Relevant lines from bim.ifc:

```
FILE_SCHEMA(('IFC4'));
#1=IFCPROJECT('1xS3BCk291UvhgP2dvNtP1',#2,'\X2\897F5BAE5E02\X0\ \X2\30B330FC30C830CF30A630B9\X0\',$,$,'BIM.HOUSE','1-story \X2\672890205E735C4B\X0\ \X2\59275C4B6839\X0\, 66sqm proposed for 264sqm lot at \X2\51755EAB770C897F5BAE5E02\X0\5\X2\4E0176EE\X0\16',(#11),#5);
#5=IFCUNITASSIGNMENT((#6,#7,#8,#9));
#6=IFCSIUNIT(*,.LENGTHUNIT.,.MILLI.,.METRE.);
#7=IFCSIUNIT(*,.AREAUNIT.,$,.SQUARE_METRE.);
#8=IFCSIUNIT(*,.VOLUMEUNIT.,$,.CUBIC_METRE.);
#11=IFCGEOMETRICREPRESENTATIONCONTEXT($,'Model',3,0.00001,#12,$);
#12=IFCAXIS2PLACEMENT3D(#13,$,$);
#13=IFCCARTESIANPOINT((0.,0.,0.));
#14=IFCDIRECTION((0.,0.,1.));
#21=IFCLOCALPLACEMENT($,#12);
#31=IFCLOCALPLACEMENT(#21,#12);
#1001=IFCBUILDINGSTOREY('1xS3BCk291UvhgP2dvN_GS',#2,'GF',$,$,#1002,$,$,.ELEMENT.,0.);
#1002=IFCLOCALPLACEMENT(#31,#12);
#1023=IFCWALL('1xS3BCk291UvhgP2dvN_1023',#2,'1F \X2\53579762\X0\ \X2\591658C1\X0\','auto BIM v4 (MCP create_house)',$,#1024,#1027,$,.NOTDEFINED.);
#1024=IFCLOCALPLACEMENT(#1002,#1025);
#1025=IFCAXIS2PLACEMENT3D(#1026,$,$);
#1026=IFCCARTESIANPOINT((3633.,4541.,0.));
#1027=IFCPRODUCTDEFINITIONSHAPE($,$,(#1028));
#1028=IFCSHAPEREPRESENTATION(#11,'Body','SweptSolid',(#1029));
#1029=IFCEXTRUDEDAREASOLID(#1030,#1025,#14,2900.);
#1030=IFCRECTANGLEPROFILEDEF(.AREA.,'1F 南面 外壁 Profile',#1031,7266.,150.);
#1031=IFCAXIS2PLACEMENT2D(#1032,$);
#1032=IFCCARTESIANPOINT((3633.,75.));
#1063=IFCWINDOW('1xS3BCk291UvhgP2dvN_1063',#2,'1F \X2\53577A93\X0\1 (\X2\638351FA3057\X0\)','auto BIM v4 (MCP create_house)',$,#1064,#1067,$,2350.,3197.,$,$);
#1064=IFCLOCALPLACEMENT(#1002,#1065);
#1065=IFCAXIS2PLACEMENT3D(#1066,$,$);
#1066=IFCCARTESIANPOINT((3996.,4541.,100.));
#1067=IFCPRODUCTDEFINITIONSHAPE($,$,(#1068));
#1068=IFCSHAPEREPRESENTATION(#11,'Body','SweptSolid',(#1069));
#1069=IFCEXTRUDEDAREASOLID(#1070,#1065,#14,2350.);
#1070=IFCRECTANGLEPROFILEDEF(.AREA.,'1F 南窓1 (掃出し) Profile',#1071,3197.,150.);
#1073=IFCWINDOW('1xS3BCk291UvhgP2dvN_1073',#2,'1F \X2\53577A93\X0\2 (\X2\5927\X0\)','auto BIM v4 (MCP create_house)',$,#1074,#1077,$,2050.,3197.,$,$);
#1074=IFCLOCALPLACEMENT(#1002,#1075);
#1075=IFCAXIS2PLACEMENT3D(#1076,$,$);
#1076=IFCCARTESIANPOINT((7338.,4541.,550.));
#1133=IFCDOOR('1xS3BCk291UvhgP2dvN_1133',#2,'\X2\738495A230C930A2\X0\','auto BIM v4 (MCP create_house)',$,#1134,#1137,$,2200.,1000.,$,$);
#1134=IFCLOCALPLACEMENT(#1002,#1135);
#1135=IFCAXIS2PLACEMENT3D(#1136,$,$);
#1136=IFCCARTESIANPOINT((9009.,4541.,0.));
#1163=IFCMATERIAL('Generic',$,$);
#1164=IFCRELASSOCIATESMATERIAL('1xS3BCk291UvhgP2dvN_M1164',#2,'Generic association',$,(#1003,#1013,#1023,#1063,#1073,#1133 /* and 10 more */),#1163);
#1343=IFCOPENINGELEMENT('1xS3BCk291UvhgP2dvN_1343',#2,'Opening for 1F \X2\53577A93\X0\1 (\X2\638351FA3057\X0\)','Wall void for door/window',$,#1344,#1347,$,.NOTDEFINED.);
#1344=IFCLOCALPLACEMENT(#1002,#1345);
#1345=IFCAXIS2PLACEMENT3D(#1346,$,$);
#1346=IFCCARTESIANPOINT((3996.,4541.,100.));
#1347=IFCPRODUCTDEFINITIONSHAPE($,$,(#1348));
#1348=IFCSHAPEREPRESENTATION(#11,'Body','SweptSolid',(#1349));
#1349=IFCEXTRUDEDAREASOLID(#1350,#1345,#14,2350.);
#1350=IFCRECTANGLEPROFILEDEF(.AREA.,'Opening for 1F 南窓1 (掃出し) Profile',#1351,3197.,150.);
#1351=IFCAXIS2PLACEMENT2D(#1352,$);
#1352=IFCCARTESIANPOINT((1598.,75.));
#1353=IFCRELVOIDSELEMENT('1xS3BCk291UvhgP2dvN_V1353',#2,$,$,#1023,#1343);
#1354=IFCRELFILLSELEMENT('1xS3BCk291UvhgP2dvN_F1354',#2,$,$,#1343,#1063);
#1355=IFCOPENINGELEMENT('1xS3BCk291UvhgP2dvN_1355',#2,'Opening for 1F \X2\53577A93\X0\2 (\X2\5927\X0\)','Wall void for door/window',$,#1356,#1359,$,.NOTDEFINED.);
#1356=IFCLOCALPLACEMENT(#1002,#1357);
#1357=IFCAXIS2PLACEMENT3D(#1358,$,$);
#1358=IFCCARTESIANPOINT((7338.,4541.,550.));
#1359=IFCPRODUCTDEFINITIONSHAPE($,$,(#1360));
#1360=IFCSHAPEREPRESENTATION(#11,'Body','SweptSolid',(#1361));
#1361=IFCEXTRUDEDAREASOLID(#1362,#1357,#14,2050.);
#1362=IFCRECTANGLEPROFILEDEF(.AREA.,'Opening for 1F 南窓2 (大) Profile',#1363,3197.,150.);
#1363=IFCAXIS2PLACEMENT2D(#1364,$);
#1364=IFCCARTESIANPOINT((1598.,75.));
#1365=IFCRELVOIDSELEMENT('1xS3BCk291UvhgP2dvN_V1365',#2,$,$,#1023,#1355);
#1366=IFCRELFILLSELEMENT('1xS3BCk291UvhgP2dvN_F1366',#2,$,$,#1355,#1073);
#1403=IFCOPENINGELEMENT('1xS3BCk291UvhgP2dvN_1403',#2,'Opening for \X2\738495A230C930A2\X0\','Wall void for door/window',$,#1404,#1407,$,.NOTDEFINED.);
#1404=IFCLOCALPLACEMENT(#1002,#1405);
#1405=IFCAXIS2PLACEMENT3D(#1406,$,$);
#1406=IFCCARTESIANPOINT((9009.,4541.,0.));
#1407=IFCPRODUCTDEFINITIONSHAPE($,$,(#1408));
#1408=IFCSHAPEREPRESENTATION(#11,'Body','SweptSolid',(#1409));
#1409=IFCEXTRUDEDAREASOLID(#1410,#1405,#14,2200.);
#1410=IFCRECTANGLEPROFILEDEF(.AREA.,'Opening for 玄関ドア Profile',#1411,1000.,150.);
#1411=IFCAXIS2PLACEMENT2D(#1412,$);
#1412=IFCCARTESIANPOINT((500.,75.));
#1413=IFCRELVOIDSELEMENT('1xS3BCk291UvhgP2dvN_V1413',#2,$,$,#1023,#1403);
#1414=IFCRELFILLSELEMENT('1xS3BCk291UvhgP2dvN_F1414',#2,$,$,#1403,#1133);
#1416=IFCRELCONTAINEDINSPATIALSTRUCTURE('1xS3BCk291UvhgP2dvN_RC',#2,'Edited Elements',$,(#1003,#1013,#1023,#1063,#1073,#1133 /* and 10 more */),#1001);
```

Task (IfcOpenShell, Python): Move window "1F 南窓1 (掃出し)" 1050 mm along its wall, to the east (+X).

```python
import ifcopenshell
import ifcopenshell.api.geometry
import ifcopenshell.util.placement

model = ifcopenshell.open("bim.ifc")

window = model.by_guid("1xS3BCk291UvhgP2dvN_1063")
opening = window.FillsVoids[0].RelatingOpeningElement
wall = opening.VoidsElements[0].RelatingBuildingElement

wall_matrix = ifcopenshell.util.placement.get_local_placement(wall.ObjectPlacement)
shift = wall_matrix[:3, 0] * 1050.0
before = ifcopenshell.util.placement.get_local_placement(window.ObjectPlacement)[:3, 3].copy()

# The window is not placed relative to its opening, so move both.
for product in (opening, window):
    matrix = ifcopenshell.util.placement.get_local_placement(product.ObjectPlacement)
    matrix[:3, 3] += shift
    ifcopenshell.api.geometry.edit_object_placement(model, product=product, matrix=matrix, is_si=False)

after = ifcopenshell.util.placement.get_local_placement(window.ObjectPlacement)[:3, 3]
print("window moved by", (after - before).round(3) + 0.0)

model.write("bim_updated.ifc")
```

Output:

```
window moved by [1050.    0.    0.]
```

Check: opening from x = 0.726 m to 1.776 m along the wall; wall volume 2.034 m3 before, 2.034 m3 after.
